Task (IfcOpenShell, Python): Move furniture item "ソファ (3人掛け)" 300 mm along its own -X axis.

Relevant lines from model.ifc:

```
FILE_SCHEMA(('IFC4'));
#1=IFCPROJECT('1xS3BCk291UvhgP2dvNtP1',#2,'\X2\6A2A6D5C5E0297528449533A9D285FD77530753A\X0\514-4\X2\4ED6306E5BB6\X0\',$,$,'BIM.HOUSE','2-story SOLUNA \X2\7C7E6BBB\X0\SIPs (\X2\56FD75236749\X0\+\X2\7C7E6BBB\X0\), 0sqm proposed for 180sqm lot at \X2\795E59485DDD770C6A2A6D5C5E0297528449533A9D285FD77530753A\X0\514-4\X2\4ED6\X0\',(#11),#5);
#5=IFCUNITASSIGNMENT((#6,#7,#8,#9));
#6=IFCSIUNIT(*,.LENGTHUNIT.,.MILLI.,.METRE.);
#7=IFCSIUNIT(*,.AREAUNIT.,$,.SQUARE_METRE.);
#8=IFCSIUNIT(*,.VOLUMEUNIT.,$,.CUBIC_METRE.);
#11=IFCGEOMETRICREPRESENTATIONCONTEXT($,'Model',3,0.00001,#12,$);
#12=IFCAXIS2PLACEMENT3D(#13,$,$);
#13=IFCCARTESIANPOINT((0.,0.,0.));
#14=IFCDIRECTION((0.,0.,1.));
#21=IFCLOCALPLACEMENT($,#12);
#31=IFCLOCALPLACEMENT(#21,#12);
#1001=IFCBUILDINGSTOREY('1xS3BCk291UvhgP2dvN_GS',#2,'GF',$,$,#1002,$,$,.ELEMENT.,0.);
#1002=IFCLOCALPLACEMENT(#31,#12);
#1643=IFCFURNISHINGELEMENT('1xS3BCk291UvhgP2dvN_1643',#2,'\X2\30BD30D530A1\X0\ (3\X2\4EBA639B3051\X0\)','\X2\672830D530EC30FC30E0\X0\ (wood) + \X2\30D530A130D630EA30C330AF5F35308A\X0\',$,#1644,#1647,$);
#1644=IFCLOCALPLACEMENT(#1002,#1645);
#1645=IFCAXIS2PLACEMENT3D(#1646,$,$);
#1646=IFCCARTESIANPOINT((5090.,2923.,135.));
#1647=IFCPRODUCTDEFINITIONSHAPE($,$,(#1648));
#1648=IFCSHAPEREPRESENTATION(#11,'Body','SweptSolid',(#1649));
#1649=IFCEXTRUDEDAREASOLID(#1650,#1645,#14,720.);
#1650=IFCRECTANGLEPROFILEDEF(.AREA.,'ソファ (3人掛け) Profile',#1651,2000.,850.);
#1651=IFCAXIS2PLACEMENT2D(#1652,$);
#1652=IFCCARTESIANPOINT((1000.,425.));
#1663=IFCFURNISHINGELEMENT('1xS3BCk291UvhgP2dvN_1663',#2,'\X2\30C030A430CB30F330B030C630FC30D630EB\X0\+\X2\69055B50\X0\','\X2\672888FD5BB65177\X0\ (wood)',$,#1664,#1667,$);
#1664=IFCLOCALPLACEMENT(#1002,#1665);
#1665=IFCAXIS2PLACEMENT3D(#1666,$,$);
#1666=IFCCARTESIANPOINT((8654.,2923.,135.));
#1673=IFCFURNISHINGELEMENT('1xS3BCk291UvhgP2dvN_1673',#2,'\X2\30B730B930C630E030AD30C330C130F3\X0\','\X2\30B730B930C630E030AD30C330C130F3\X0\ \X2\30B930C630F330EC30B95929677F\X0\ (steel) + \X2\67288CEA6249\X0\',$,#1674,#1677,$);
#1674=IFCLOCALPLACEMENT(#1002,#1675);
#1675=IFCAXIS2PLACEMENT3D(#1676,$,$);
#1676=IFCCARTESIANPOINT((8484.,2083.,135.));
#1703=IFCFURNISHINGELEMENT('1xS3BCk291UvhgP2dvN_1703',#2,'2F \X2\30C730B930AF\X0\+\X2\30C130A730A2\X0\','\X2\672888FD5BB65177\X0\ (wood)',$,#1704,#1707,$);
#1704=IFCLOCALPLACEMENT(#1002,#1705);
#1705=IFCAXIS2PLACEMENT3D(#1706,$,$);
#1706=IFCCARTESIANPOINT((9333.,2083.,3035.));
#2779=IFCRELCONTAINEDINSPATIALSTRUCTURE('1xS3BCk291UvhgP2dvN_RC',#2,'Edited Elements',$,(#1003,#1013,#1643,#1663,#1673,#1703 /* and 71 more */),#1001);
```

```python
import ifcopenshell
import ifcopenshell.api.geometry
import ifcopenshell.util.placement
import ifcopenshell.util.unit

model = ifcopenshell.open("model.ifc")
unit_scale = ifcopenshell.util.unit.calculate_unit_scale(model)

item = model.by_id(1643)
matrix = ifcopenshell.util.placement.get_local_placement(item.ObjectPlacement)
matrix[:3, 3] -= matrix[:3, 0] * 0.3 / unit_scale
ifcopenshell.api.geometry.edit_object_placement(model, product=item, matrix=matrix, is_si=False)

print(ifcopenshell.util.placement.get_local_placement(item.ObjectPlacement).round(3) + 0.0)

model.write("model_edited.ifc")
```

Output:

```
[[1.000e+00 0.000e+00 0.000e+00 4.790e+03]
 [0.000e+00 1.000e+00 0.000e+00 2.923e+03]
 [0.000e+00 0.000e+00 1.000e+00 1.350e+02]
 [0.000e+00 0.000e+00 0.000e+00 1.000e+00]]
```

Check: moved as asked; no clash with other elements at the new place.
